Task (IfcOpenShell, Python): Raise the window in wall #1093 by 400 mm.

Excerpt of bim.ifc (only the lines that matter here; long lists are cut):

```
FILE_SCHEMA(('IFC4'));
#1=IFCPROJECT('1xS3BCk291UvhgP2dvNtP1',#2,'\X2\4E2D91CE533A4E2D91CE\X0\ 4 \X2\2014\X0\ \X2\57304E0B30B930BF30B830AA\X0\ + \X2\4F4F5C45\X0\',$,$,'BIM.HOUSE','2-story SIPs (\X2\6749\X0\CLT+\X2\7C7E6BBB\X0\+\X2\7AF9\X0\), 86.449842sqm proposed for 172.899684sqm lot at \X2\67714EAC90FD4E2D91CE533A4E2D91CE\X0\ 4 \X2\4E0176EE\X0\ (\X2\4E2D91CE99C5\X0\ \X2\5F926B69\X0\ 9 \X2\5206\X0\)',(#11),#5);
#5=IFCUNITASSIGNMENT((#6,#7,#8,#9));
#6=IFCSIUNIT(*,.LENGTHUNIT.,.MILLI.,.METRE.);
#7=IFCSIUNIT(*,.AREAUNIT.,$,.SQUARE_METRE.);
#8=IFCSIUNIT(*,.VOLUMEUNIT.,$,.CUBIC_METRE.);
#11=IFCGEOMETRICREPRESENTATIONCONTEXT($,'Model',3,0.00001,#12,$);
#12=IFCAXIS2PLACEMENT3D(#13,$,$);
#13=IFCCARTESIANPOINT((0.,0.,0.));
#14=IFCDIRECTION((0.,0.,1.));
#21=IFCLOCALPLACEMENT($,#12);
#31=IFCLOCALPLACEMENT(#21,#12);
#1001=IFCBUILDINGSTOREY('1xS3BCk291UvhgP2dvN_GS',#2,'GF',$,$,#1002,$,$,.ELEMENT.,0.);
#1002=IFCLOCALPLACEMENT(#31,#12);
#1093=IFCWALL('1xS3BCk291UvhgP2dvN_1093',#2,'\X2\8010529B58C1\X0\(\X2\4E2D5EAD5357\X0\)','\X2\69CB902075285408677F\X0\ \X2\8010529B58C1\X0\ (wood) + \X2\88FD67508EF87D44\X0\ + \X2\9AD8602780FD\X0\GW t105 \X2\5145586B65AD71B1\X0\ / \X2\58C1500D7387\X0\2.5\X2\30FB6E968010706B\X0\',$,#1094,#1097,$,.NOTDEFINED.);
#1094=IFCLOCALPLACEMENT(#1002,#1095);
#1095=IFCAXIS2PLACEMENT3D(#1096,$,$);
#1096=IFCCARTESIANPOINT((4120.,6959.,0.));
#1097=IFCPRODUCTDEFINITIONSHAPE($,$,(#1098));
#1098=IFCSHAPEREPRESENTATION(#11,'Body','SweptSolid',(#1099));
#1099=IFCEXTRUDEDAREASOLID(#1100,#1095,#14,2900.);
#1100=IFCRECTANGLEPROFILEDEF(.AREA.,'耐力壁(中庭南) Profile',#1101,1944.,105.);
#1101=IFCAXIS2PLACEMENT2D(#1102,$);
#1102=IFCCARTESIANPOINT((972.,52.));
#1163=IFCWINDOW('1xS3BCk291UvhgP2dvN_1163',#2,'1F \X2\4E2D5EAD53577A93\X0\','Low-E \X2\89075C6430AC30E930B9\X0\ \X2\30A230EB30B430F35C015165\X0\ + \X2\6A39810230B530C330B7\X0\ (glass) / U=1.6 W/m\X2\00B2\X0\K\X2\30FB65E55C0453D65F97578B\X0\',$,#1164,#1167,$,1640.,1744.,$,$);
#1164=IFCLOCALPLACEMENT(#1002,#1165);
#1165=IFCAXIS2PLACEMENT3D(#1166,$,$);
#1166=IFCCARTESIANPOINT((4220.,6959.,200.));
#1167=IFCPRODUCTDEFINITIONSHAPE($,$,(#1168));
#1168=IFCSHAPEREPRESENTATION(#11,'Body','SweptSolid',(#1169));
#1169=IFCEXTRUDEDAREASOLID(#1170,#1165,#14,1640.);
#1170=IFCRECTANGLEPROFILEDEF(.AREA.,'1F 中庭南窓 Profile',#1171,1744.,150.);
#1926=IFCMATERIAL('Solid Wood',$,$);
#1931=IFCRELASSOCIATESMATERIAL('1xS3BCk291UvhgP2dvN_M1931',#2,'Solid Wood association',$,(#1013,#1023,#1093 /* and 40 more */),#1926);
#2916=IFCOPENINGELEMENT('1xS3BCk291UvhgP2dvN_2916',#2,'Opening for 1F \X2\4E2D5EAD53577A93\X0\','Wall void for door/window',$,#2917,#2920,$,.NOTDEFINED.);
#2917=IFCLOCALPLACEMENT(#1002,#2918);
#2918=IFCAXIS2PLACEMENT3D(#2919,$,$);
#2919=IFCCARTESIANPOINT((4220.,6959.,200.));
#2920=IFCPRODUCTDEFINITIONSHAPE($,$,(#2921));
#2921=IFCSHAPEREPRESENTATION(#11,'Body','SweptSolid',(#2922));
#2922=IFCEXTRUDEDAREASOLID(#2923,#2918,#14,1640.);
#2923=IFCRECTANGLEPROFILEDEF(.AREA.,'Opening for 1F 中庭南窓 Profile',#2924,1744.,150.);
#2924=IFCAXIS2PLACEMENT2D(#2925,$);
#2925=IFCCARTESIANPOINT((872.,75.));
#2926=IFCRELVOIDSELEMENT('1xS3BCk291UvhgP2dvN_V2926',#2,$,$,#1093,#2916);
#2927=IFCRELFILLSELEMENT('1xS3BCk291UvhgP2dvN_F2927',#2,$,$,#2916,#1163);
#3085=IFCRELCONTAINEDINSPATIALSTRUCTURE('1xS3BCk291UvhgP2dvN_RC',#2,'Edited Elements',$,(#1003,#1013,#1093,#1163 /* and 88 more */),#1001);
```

```python
import numpy as np
import ifcopenshell
import ifcopenshell.api.geometry
import ifcopenshell.util.placement
import ifcopenshell.util.unit

model = ifcopenshell.open("bim.ifc")
unit_scale = ifcopenshell.util.unit.calculate_unit_scale(model)

window = model.by_guid("1xS3BCk291UvhgP2dvN_1163")
opening = window.FillsVoids[0].RelatingOpeningElement
dz = 400.0

shift = np.array([0.0, 0.0, dz])
# The window is not placed relative to its opening, so move both.
for product in (opening, window):
    matrix = ifcopenshell.util.placement.get_local_placement(product.ObjectPlacement)
    matrix[:3, 3] += shift
    ifcopenshell.api.geometry.edit_object_placement(model, product=product, matrix=matrix, is_si=False)

print(f"moved by {dz * unit_scale:+.3f} m")

model.write("bim_updated.ifc")
```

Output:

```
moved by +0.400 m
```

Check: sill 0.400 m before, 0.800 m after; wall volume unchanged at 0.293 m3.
